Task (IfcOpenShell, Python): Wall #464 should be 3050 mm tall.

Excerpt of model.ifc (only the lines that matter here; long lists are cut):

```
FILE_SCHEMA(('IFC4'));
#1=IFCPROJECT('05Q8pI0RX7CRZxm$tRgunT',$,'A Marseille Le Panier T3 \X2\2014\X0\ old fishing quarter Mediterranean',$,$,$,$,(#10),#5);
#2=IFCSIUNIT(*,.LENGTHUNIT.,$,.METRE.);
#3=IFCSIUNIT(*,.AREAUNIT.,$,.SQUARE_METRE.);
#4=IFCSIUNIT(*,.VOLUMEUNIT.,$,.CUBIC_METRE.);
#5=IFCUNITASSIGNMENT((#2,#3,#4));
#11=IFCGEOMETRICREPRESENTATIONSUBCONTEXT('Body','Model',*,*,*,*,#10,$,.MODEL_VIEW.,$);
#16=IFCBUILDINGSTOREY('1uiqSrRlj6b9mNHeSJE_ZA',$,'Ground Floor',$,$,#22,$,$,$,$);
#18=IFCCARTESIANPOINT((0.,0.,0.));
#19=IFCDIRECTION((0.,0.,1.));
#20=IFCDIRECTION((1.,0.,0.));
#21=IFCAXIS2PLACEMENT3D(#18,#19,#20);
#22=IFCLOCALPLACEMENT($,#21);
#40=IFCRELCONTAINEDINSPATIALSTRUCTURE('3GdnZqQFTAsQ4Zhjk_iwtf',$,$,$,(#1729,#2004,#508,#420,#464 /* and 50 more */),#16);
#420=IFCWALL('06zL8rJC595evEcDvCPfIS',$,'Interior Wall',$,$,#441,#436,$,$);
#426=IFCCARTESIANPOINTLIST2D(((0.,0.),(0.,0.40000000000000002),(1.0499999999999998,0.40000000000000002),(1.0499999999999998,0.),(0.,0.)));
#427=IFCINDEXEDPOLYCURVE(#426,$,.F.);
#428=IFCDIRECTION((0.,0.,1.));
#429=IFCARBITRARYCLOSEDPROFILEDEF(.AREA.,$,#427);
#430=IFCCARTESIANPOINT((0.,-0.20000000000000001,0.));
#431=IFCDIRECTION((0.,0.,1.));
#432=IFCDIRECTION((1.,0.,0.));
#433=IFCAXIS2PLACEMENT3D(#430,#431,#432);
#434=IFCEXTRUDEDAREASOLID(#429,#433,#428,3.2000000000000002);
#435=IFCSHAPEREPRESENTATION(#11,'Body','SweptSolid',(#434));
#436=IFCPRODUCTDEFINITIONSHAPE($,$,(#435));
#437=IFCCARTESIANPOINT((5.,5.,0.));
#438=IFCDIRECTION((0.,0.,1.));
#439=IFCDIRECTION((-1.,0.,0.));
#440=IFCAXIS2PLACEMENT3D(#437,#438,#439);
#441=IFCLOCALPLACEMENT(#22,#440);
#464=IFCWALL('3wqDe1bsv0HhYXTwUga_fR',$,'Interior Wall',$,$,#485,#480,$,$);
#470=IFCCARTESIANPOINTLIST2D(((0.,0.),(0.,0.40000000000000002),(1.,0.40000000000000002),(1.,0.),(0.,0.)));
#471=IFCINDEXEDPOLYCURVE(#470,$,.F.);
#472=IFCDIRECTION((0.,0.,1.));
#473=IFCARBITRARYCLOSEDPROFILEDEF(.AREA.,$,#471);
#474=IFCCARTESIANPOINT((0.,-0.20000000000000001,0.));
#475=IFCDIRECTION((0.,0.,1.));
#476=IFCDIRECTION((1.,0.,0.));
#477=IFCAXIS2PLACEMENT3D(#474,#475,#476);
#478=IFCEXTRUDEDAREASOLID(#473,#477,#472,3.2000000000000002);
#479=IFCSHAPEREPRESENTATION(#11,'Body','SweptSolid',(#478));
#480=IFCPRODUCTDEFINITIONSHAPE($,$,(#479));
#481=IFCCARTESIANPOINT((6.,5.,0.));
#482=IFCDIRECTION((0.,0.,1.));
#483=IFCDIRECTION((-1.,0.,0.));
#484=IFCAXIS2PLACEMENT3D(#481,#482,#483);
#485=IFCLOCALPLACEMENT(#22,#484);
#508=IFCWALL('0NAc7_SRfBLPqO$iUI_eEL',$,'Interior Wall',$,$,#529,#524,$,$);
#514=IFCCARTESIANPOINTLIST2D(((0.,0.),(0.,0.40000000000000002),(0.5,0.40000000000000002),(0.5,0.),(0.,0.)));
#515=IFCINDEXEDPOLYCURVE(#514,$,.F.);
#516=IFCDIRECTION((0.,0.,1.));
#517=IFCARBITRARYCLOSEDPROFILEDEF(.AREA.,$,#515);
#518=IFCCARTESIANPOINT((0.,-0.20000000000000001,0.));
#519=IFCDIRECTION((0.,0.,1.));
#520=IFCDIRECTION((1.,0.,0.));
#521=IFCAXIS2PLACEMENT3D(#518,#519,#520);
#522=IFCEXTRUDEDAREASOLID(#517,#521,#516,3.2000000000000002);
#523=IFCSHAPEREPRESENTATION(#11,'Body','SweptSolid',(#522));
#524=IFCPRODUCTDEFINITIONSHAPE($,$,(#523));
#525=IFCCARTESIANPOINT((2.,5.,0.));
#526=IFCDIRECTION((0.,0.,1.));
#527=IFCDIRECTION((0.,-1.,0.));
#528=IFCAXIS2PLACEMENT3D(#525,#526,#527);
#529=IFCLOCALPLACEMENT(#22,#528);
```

```python
import ifcopenshell
import ifcopenshell.geom
import ifcopenshell.util.representation
import ifcopenshell.util.shape

model = ifcopenshell.open("model.ifc")
settings = ifcopenshell.geom.settings()


def volume(element):
    """Net volume in cubic metres, openings subtracted."""
    shape = ifcopenshell.geom.create_shape(settings, element)
    return ifcopenshell.util.shape.get_volume(shape.geometry)


wall = model.by_id(464)
before = volume(wall)

body = ifcopenshell.util.representation.get_representation(wall, "Model", "Body")
solid = body.Items[0]
old_height = solid.Depth
solid.Depth = 3.05
after = volume(wall)

print(f"height {old_height:g} -> {solid.Depth:g}, volume {before:.3f} -> {after:.3f} m3")

model.write("model_rev.ifc")
```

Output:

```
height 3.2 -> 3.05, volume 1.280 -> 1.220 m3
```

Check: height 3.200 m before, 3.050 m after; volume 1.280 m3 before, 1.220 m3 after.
